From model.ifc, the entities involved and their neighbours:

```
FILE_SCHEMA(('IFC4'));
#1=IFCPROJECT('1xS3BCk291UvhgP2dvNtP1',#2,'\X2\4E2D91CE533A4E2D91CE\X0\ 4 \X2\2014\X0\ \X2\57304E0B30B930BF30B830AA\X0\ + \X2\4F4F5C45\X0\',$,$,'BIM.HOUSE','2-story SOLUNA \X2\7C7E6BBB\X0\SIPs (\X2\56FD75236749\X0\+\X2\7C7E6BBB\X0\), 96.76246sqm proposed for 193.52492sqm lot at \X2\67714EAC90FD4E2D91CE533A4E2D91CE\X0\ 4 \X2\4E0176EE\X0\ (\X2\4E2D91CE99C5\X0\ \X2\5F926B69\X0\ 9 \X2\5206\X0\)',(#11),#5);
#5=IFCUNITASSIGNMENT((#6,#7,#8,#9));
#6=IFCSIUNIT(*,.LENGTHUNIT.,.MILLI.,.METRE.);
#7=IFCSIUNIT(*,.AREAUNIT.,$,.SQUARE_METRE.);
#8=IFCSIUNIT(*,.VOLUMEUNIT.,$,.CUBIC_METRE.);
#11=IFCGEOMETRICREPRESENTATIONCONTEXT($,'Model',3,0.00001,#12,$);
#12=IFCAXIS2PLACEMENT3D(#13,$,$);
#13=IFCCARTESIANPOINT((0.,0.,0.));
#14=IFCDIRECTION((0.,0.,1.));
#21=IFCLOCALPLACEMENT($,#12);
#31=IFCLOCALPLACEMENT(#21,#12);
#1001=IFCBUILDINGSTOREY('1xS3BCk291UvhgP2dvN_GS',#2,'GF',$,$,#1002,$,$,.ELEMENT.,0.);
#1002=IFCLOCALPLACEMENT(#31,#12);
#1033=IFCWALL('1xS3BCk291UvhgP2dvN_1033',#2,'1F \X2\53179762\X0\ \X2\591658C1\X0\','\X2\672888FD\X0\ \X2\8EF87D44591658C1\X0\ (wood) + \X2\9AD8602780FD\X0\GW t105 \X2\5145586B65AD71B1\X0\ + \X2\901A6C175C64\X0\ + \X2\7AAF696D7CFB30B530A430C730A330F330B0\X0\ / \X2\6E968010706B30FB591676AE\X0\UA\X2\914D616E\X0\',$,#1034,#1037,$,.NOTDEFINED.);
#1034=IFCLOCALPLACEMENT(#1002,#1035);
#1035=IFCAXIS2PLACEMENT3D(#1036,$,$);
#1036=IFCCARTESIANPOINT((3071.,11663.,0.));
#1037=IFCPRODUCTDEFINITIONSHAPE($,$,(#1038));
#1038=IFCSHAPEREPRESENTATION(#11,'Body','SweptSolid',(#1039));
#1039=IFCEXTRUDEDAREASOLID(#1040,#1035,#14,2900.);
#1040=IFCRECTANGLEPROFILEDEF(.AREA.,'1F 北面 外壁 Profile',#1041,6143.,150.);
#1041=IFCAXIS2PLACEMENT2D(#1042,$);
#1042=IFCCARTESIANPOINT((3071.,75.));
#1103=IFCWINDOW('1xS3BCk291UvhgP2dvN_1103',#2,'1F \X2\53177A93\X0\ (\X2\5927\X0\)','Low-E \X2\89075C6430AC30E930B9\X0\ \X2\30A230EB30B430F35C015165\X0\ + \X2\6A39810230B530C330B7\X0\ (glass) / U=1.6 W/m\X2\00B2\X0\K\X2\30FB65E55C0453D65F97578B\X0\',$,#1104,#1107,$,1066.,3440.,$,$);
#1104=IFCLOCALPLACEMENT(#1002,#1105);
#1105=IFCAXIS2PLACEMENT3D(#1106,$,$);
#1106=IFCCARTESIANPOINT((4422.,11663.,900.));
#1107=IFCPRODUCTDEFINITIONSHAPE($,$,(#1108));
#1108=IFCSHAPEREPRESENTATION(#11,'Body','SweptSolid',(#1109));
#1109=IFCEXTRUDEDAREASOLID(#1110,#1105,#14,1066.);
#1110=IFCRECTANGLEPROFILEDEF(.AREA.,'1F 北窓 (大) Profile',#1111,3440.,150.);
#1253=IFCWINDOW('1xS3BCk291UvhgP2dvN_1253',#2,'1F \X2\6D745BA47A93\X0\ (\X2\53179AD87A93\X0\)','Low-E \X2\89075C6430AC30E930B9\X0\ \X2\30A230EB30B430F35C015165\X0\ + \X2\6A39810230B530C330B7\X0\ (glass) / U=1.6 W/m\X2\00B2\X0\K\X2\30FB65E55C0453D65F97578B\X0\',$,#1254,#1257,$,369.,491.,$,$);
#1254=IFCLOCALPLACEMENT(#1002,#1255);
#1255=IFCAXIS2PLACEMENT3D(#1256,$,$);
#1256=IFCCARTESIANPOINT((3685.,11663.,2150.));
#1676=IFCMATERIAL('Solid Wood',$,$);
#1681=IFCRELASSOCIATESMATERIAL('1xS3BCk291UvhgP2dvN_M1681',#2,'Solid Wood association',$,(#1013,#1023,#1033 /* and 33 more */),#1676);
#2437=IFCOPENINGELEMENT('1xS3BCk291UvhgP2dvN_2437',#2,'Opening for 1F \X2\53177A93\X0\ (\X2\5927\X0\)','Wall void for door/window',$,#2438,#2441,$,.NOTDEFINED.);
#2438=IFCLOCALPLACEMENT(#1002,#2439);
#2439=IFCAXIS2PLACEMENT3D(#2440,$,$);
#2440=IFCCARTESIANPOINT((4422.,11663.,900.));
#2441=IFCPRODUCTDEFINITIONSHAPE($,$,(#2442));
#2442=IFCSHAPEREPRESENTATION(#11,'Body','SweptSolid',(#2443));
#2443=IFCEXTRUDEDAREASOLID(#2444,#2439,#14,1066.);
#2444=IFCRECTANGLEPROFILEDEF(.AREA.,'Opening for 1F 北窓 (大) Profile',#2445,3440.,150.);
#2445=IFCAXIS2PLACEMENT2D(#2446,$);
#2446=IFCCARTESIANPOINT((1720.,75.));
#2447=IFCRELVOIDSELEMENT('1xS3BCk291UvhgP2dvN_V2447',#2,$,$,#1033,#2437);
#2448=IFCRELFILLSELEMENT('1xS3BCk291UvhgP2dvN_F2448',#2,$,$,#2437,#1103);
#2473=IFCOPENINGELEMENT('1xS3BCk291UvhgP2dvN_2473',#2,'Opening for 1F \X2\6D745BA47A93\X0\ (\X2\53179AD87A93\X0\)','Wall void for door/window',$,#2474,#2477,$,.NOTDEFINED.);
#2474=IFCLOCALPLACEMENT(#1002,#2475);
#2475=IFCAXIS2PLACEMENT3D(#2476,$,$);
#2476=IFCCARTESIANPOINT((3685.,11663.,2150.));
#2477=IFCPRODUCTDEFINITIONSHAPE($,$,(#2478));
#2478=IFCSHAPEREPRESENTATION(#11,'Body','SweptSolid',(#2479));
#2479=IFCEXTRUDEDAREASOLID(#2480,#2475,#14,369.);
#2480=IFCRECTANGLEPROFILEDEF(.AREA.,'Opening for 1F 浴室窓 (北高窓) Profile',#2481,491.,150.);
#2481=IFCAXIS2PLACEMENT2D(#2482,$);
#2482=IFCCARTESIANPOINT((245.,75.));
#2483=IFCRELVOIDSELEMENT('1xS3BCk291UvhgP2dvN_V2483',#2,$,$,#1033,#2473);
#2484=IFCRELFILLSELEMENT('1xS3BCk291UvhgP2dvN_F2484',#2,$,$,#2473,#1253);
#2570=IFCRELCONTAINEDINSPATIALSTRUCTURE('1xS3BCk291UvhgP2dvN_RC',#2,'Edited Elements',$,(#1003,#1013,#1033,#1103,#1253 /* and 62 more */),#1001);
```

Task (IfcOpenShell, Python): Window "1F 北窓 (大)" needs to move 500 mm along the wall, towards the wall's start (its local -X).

```python
import ifcopenshell
import ifcopenshell.api.geometry
import ifcopenshell.util.placement
import ifcopenshell.util.unit

model = ifcopenshell.open("model.ifc")
unit_scale = ifcopenshell.util.unit.calculate_unit_scale(model)

window = model.by_guid("1xS3BCk291UvhgP2dvN_1103")
opening = window.FillsVoids[0].RelatingOpeningElement
wall = opening.VoidsElements[0].RelatingBuildingElement

wall_matrix = ifcopenshell.util.placement.get_local_placement(wall.ObjectPlacement)
shift = wall_matrix[:3, 0] * -0.5 / unit_scale
before = ifcopenshell.util.placement.get_local_placement(window.ObjectPlacement)[:3, 3].copy()

# The window is not placed relative to its opening, so move both.
for product in (opening, window):
    matrix = ifcopenshell.util.placement.get_local_placement(product.ObjectPlacement)
    matrix[:3, 3] += shift
    ifcopenshell.api.geometry.edit_object_placement(model, product=product, matrix=matrix, is_si=False)

after = ifcopenshell.util.placement.get_local_placement(window.ObjectPlacement)[:3, 3]
print("window moved by", (after - before).round(3) + 0.0)

model.write("model_v2.ifc")
```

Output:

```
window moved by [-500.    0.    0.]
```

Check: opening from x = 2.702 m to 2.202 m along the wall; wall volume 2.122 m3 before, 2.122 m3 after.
